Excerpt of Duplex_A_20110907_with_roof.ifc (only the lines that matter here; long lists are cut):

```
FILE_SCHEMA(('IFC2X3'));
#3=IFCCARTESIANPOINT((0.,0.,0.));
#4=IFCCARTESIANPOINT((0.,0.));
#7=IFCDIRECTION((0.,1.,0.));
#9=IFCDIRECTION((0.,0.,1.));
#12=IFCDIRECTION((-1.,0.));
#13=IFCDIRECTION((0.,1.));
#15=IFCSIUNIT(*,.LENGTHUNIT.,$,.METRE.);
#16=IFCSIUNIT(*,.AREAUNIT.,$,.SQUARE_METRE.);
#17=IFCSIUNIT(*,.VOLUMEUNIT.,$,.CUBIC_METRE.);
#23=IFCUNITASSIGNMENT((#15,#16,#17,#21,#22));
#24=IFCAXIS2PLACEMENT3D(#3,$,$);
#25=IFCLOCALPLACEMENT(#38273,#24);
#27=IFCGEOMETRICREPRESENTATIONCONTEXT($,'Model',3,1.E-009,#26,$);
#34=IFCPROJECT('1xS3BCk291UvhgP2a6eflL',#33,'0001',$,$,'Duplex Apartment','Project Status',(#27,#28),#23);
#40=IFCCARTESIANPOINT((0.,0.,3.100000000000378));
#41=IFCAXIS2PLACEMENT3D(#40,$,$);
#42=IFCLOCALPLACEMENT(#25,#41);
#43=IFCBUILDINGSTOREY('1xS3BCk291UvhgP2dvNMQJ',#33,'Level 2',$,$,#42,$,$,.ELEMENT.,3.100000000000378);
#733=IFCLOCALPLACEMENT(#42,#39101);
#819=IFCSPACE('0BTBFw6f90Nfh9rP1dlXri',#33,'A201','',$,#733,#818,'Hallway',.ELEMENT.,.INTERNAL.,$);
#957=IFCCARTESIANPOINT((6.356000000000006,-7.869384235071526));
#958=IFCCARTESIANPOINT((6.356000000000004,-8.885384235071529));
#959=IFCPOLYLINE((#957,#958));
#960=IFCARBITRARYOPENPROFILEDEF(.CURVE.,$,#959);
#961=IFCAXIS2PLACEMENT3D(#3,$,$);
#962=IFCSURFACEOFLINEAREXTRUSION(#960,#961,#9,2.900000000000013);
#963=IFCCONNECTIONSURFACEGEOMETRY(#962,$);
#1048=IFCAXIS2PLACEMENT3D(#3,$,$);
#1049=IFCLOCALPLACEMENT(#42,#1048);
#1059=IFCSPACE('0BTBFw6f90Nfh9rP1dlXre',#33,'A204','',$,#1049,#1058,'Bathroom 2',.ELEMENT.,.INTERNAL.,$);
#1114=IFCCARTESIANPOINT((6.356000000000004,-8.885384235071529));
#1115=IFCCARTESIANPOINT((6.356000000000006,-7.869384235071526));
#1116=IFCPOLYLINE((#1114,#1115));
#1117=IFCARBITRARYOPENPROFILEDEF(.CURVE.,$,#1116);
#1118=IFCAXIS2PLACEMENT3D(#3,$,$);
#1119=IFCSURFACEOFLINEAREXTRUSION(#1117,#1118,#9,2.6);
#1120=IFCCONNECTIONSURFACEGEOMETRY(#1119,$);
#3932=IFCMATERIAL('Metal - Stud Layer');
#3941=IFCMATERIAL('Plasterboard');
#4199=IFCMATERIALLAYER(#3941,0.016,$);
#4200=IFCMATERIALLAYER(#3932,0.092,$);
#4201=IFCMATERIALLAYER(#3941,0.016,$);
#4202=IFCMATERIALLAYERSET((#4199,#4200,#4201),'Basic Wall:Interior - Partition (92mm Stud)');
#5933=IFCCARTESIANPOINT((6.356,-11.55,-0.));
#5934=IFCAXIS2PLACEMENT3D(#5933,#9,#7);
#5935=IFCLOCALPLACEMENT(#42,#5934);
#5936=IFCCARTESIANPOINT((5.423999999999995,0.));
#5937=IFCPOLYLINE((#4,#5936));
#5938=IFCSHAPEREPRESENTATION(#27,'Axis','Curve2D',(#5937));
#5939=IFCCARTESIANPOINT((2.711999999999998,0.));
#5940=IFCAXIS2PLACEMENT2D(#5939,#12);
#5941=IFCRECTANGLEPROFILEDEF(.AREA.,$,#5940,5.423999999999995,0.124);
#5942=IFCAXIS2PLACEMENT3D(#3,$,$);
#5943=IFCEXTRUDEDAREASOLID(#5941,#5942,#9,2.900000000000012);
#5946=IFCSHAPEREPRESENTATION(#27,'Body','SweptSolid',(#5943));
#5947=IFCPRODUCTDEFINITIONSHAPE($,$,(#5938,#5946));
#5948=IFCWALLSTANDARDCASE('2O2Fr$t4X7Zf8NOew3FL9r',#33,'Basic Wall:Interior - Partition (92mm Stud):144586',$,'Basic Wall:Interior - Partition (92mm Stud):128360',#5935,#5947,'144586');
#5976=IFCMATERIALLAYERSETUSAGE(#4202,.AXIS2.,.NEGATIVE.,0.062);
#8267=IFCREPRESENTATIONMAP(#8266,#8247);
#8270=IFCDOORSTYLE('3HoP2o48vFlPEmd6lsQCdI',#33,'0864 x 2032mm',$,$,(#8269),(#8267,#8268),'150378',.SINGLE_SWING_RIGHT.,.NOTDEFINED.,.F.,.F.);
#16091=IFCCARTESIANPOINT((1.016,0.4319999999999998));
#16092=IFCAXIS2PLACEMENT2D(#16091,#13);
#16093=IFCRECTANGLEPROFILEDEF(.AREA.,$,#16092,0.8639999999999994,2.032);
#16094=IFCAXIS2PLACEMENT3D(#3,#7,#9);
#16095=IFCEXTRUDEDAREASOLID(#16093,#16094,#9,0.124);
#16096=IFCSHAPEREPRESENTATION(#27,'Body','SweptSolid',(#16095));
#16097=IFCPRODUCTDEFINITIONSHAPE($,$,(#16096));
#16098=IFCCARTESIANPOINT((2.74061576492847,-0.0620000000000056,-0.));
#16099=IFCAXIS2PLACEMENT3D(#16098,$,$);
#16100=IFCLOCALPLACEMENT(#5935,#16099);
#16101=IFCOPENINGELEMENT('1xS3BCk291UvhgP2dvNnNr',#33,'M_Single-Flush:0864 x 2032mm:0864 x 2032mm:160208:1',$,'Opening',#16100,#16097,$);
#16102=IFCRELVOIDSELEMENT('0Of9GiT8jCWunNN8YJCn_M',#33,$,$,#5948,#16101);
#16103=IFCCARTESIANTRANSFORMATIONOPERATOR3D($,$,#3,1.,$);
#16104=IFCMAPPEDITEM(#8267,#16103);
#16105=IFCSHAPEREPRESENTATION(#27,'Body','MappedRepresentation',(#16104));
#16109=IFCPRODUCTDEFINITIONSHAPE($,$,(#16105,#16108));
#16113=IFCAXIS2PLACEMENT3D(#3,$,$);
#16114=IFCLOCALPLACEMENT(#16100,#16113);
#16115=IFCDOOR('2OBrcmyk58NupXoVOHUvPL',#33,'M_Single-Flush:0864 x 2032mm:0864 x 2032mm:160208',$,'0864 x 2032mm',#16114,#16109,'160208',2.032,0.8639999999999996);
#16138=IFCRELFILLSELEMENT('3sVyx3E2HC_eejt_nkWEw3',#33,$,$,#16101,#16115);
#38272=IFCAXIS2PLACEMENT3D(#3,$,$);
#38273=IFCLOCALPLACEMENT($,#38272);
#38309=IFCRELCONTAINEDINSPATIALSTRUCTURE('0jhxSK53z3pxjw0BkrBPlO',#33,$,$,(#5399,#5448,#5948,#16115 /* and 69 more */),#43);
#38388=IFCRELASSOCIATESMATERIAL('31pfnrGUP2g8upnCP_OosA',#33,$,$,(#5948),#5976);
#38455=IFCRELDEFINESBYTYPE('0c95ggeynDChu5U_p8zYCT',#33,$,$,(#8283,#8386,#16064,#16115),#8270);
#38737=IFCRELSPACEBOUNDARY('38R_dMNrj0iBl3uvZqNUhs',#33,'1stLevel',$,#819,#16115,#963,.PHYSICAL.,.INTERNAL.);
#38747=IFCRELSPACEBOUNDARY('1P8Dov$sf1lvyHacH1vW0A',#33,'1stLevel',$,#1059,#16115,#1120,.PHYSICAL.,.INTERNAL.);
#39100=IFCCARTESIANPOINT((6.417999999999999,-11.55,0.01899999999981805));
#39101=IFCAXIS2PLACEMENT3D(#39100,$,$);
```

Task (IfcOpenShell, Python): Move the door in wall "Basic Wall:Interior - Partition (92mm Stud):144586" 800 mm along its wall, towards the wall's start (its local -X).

```python
import numpy as np
import ifcopenshell
import ifcopenshell.api.geometry
import ifcopenshell.util.placement
import ifcopenshell.util.unit

model = ifcopenshell.open("Duplex_A_20110907_with_roof.ifc")
unit_scale = ifcopenshell.util.unit.calculate_unit_scale(model)

door = model.by_guid("2OBrcmyk58NupXoVOHUvPL")
opening = door.FillsVoids[0].RelatingOpeningElement
wall = opening.VoidsElements[0].RelatingBuildingElement

wall_matrix = ifcopenshell.util.placement.get_local_placement(wall.ObjectPlacement)
shift = wall_matrix[:3, 0] * -0.8 / unit_scale
before = ifcopenshell.util.placement.get_local_placement(door.ObjectPlacement)[:3, 3].copy()

# The door is placed relative to its opening, so it follows when the opening moves.
matrix = ifcopenshell.util.placement.get_local_placement(opening.ObjectPlacement)
matrix[:3, 3] += shift
ifcopenshell.api.geometry.edit_object_placement(
    model, product=opening, matrix=matrix, is_si=False, should_transform_children=True
)

# Space boundary surfaces are stored in each space's coordinates; move them too.
for rel in door.ProvidesBoundaries:
    if not rel.ConnectionGeometry:
        continue
    surface = rel.ConnectionGeometry.SurfaceOnRelatingElement
    space_matrix = ifcopenshell.util.placement.get_local_placement(rel.RelatingSpace.ObjectPlacement)
    point = np.array(surface.Position.Location.Coordinates) + space_matrix[:3, :3].T @ shift
    surface.Position = model.createIfcAxis2Placement3D(
        model.createIfcCartesianPoint(point.tolist()), surface.Position.Axis, surface.Position.RefDirection
    )

after = ifcopenshell.util.placement.get_local_placement(door.ObjectPlacement)[:3, 3]
print("door moved by", (after - before).round(3) + 0.0)

model.write("Duplex_A_20110907_with_roof-out.ifc")
```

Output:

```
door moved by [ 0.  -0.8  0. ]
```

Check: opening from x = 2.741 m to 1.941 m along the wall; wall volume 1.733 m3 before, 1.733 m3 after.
